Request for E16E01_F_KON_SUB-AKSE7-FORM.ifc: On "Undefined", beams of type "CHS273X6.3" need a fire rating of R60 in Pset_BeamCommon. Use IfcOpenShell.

First a look at what the model holds.

```python
import ifcopenshell
import ifcopenshell.util.element

model = ifcopenshell.open("E16E01_F_KON_SUB-AKSE7-FORM.ifc")
print(model.schema)
storey = next(s for s in model.by_type("IfcBuildingStorey") if s.Name == "Undefined")
beams = [e for e in ifcopenshell.util.element.get_decomposition(storey) if e.is_a("IfcBeam")]
seen = {}
for e in beams:
    element_type = ifcopenshell.util.element.get_type(e)
    key = (element_type.Name if element_type != e and element_type else None, ifcopenshell.util.element.get_pset(e, "Pset_BeamCommon", "FireRating"))
    seen[key] = seen.get(key, 0) + 1
for (name, value), count in sorted(seen.items(), key=str):
    print(count, "x", name, "|", value)
```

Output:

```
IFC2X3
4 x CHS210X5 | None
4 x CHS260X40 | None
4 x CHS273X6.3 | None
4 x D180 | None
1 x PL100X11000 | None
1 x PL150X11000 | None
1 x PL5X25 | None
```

```python
import ifcopenshell
import ifcopenshell.api.pset
import ifcopenshell.util.element

model = ifcopenshell.open("E16E01_F_KON_SUB-AKSE7-FORM.ifc")

storey = next(s for s in model.by_type("IfcBuildingStorey") if s.Name == "Undefined")
beams = [e for e in ifcopenshell.util.element.get_decomposition(storey) if e.is_a("IfcBeam")]

count = 0
for e in beams:
    element_type = ifcopenshell.util.element.get_type(e)
    if element_type in (None, e) or element_type.Name != "CHS273X6.3":
        continue
    found = ifcopenshell.util.element.get_pset(e, "Pset_BeamCommon", should_inherit=False)
    if found:
        pset = model.by_id(found["id"])
        if len(ifcopenshell.util.element.get_elements_by_pset(pset)) > 1:
            pset = ifcopenshell.api.pset.unshare_pset(model, products=[e], pset=pset)[0]
    else:
        pset = ifcopenshell.api.pset.add_pset(model, product=e, name="Pset_BeamCommon")
    ifcopenshell.api.pset.edit_pset(model, pset=pset, properties={"FireRating": "R60"})
    count += 1

print(count, "beams updated")

model.write("E16E01_F_KON_SUB-AKSE7-FORM_edited.ifc")
```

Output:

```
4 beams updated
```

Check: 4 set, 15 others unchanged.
